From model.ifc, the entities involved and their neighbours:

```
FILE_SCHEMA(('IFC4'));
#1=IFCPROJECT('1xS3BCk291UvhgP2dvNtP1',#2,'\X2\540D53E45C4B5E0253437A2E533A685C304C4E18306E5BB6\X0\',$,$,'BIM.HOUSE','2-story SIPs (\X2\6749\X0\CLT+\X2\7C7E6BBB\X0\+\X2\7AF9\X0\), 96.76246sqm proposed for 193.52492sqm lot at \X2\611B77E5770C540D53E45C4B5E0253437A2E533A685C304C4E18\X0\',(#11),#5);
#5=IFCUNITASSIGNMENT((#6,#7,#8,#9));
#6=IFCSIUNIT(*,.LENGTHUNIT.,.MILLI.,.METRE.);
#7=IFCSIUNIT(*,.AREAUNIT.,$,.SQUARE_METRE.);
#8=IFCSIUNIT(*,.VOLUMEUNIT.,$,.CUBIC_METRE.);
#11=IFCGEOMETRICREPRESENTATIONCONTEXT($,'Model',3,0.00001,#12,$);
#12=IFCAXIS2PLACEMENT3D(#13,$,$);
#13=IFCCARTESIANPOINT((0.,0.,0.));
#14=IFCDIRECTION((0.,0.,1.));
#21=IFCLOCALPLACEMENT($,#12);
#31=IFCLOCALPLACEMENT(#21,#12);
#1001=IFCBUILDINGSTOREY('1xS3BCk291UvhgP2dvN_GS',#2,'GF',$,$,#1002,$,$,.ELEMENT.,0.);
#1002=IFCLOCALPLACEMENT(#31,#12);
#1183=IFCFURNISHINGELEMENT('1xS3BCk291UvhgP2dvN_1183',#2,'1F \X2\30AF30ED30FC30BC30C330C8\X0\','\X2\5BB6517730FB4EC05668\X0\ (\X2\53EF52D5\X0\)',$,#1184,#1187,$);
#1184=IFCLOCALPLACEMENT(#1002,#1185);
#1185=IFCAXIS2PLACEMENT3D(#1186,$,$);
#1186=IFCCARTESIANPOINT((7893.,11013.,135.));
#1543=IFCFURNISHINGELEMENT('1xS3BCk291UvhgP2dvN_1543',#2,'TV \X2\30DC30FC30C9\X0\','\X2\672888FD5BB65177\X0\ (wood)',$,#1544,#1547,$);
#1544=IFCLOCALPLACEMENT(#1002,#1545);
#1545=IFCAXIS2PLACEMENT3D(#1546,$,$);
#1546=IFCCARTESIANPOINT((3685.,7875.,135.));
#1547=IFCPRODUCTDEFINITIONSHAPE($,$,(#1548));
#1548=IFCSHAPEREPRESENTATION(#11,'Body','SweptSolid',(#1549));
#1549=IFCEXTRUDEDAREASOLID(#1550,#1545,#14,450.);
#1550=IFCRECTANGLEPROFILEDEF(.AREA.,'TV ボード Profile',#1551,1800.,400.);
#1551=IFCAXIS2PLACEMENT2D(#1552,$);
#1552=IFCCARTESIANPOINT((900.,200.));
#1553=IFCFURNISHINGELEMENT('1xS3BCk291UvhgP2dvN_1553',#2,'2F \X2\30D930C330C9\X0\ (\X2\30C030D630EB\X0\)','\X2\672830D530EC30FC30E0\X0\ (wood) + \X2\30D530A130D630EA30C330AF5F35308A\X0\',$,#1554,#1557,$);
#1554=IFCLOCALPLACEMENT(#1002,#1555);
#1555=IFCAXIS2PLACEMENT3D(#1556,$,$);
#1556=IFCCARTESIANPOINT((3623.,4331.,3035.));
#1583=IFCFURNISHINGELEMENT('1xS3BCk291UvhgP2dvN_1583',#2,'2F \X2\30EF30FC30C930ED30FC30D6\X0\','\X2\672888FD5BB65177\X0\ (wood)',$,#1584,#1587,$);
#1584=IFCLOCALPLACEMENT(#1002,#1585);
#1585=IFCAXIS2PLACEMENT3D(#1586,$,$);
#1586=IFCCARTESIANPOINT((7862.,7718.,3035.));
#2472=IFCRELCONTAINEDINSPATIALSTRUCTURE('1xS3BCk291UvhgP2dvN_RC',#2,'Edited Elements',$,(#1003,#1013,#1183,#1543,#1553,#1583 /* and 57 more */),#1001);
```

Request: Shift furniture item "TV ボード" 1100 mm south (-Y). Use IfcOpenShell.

```python
import ifcopenshell
import ifcopenshell.api.geometry
import ifcopenshell.util.placement

model = ifcopenshell.open("model.ifc")

item = model.by_guid("1xS3BCk291UvhgP2dvN_1543")
matrix = ifcopenshell.util.placement.get_local_placement(item.ObjectPlacement)
matrix[1, 3] -= 1100.0
ifcopenshell.api.geometry.edit_object_placement(model, product=item, matrix=matrix, is_si=False)

print(ifcopenshell.util.placement.get_local_placement(item.ObjectPlacement).round(3) + 0.0)

model.write("model-out.ifc")
```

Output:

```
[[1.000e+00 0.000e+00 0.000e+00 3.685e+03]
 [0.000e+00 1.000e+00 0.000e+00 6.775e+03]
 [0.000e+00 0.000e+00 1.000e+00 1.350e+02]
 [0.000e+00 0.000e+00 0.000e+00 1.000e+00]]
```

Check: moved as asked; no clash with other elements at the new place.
